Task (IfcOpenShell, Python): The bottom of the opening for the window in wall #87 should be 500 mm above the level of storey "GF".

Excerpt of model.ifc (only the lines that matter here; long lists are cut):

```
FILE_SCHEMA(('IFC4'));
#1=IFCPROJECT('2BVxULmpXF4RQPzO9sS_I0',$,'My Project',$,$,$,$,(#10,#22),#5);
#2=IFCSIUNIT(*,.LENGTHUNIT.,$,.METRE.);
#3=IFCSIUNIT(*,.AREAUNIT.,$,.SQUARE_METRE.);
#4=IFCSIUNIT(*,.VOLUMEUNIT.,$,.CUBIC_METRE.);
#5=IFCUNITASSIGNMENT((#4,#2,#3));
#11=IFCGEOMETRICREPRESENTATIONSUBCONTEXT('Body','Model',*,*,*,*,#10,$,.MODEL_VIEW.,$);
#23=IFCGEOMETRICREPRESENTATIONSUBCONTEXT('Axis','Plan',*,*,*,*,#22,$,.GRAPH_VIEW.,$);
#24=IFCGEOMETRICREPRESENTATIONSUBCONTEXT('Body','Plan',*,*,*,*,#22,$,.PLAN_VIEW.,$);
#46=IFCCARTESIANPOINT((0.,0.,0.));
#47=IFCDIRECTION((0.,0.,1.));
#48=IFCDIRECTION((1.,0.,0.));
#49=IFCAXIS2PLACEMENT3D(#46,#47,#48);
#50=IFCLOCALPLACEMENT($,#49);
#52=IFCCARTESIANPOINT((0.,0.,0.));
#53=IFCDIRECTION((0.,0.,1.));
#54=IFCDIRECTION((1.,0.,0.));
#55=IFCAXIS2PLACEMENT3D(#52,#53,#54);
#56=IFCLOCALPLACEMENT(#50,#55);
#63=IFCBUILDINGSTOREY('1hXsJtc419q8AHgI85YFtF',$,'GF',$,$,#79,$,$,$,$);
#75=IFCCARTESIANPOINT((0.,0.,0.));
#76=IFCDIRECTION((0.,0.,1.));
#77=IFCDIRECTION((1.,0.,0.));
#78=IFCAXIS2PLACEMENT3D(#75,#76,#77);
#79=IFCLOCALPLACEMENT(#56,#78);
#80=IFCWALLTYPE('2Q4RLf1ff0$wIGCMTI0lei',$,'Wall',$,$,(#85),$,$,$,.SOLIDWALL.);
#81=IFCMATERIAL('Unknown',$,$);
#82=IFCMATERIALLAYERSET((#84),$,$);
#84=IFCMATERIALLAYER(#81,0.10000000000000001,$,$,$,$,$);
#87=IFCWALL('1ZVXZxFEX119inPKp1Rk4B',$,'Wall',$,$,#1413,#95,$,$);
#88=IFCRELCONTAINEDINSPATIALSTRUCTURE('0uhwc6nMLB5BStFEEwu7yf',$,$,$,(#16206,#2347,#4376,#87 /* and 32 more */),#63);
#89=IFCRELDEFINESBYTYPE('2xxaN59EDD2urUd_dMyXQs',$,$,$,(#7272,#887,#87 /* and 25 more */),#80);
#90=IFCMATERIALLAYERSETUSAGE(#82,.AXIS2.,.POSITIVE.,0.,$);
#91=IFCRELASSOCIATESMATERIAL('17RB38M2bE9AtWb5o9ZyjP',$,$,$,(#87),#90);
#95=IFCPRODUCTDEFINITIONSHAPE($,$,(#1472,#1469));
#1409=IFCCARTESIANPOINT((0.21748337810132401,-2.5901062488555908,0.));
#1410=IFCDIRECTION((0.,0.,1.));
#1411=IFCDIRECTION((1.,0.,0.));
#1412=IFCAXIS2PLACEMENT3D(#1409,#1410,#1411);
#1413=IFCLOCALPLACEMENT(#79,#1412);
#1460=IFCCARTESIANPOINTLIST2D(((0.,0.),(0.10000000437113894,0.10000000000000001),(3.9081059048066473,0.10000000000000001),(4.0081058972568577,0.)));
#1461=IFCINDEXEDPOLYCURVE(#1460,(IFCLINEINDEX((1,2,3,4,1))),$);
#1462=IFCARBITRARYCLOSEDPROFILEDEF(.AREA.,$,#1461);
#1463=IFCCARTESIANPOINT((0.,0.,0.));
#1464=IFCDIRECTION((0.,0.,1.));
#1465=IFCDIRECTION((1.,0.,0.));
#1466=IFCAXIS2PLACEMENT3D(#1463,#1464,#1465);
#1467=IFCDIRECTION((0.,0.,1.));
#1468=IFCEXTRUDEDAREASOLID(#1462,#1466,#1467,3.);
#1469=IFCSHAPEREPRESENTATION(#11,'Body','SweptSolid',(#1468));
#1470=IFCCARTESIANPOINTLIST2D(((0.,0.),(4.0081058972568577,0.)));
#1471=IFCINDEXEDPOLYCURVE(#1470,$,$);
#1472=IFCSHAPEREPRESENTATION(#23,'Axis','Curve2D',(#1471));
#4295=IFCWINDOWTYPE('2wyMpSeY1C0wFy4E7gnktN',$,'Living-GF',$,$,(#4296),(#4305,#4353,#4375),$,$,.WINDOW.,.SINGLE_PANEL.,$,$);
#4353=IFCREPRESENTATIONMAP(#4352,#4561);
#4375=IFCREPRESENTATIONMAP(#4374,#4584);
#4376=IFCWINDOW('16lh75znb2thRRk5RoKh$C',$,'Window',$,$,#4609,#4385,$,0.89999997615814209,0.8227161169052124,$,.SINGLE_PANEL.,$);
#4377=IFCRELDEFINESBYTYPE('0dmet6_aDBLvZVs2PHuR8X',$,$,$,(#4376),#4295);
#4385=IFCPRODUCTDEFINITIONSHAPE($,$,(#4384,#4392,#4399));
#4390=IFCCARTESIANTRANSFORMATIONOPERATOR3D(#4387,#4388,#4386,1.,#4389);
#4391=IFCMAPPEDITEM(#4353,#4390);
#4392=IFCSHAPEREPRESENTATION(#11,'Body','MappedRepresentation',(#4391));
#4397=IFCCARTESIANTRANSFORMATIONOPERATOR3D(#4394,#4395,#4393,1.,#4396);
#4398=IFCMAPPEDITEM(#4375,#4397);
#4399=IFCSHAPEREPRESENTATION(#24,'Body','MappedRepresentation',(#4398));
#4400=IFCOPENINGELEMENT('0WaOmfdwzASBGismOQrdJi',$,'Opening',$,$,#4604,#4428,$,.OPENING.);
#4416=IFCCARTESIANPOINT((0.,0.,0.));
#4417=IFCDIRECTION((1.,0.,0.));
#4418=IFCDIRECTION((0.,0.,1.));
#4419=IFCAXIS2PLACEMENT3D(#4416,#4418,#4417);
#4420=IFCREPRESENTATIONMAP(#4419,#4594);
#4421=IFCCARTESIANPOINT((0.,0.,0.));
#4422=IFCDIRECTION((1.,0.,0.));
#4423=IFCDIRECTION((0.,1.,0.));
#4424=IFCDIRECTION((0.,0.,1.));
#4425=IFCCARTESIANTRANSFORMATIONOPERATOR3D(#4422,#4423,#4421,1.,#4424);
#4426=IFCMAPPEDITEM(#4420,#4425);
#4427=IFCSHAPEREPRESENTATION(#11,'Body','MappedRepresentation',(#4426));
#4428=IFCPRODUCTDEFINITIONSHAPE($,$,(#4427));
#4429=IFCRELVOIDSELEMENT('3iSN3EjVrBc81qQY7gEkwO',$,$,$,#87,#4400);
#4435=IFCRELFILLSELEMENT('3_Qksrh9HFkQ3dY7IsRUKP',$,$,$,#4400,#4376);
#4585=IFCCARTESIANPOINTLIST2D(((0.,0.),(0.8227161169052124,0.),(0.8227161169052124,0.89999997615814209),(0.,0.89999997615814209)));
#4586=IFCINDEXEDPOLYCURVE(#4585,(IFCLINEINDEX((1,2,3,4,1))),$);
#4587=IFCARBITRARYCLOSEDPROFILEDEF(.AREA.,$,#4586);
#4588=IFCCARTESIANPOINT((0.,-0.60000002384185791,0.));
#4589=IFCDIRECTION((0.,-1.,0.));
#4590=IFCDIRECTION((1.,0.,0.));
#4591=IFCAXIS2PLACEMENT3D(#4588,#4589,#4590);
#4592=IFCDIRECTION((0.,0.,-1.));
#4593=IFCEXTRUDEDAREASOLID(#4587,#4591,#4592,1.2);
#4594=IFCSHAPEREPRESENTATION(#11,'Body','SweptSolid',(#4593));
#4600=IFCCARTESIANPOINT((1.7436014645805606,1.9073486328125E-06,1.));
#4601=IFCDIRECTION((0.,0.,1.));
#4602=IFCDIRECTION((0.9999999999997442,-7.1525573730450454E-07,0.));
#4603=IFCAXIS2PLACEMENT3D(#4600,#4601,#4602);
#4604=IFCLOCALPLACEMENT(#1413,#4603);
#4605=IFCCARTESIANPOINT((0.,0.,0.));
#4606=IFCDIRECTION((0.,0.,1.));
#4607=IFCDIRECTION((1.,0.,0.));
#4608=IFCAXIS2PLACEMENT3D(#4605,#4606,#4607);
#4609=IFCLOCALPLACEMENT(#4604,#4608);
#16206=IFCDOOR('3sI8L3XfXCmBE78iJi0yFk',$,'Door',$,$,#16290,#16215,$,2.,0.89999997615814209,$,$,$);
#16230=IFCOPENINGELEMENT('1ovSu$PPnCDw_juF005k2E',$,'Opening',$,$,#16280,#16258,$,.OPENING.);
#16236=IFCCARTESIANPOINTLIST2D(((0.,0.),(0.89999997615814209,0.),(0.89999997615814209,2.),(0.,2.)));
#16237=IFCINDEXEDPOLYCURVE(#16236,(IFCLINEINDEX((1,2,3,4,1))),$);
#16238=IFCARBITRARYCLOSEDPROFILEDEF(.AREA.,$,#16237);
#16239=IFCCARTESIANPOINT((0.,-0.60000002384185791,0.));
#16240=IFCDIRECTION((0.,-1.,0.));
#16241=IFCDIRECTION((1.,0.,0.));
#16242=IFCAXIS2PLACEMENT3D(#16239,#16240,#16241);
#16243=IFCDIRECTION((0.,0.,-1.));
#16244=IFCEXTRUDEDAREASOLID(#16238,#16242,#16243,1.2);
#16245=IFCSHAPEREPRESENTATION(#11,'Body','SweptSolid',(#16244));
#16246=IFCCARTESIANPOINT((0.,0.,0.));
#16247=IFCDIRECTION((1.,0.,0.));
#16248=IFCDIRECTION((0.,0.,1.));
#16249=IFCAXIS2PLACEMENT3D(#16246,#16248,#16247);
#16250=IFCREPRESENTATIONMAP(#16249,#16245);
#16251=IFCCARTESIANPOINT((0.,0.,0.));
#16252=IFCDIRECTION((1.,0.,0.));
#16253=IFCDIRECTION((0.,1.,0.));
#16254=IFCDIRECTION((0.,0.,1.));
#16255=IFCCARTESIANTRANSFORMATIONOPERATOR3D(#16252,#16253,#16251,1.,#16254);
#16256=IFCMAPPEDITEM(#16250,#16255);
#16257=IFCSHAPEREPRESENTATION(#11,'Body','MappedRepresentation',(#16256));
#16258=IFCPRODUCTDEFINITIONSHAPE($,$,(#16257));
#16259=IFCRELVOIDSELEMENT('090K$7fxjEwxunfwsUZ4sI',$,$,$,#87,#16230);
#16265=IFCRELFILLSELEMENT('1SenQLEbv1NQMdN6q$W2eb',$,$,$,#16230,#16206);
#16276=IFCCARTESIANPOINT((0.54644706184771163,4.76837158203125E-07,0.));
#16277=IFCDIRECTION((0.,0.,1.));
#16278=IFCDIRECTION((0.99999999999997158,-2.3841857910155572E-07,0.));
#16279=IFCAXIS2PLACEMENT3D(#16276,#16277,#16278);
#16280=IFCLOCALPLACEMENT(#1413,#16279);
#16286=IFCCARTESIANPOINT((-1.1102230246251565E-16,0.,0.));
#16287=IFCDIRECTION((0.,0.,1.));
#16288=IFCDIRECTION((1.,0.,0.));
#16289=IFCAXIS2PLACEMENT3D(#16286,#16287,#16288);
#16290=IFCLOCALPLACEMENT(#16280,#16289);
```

```python
import numpy as np
import ifcopenshell
import ifcopenshell.api.geometry
import ifcopenshell.geom
import ifcopenshell.util.element
import ifcopenshell.util.placement
import ifcopenshell.util.shape
import ifcopenshell.util.unit

model = ifcopenshell.open("model.ifc")
unit_scale = ifcopenshell.util.unit.calculate_unit_scale(model)

window = model.by_guid("16lh75znb2thRRk5RoKh$C")
opening = window.FillsVoids[0].RelatingOpeningElement
storey = ifcopenshell.util.element.get_container(window, ifc_class="IfcBuildingStorey")
level = ifcopenshell.util.placement.get_local_placement(storey.ObjectPlacement)[2, 3]

# The opening's origin need not be at the sill, so measure its lowest point.
shape = ifcopenshell.geom.create_shape(ifcopenshell.geom.settings(), opening)
bottom = ifcopenshell.util.shape.get_shape_bottom_elevation(shape, shape.geometry) / unit_scale
dz = level + 0.5 / unit_scale - bottom

shift = np.array([0.0, 0.0, dz])
# The window is placed relative to its opening, so it follows when the opening moves.
matrix = ifcopenshell.util.placement.get_local_placement(opening.ObjectPlacement)
matrix[:3, 3] += shift
ifcopenshell.api.geometry.edit_object_placement(
    model, product=opening, matrix=matrix, is_si=False, should_transform_children=True
)

print(f"moved by {dz * unit_scale:+.3f} m")

model.write("model_edited.ifc")
```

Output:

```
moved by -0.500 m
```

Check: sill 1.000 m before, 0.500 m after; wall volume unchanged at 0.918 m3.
